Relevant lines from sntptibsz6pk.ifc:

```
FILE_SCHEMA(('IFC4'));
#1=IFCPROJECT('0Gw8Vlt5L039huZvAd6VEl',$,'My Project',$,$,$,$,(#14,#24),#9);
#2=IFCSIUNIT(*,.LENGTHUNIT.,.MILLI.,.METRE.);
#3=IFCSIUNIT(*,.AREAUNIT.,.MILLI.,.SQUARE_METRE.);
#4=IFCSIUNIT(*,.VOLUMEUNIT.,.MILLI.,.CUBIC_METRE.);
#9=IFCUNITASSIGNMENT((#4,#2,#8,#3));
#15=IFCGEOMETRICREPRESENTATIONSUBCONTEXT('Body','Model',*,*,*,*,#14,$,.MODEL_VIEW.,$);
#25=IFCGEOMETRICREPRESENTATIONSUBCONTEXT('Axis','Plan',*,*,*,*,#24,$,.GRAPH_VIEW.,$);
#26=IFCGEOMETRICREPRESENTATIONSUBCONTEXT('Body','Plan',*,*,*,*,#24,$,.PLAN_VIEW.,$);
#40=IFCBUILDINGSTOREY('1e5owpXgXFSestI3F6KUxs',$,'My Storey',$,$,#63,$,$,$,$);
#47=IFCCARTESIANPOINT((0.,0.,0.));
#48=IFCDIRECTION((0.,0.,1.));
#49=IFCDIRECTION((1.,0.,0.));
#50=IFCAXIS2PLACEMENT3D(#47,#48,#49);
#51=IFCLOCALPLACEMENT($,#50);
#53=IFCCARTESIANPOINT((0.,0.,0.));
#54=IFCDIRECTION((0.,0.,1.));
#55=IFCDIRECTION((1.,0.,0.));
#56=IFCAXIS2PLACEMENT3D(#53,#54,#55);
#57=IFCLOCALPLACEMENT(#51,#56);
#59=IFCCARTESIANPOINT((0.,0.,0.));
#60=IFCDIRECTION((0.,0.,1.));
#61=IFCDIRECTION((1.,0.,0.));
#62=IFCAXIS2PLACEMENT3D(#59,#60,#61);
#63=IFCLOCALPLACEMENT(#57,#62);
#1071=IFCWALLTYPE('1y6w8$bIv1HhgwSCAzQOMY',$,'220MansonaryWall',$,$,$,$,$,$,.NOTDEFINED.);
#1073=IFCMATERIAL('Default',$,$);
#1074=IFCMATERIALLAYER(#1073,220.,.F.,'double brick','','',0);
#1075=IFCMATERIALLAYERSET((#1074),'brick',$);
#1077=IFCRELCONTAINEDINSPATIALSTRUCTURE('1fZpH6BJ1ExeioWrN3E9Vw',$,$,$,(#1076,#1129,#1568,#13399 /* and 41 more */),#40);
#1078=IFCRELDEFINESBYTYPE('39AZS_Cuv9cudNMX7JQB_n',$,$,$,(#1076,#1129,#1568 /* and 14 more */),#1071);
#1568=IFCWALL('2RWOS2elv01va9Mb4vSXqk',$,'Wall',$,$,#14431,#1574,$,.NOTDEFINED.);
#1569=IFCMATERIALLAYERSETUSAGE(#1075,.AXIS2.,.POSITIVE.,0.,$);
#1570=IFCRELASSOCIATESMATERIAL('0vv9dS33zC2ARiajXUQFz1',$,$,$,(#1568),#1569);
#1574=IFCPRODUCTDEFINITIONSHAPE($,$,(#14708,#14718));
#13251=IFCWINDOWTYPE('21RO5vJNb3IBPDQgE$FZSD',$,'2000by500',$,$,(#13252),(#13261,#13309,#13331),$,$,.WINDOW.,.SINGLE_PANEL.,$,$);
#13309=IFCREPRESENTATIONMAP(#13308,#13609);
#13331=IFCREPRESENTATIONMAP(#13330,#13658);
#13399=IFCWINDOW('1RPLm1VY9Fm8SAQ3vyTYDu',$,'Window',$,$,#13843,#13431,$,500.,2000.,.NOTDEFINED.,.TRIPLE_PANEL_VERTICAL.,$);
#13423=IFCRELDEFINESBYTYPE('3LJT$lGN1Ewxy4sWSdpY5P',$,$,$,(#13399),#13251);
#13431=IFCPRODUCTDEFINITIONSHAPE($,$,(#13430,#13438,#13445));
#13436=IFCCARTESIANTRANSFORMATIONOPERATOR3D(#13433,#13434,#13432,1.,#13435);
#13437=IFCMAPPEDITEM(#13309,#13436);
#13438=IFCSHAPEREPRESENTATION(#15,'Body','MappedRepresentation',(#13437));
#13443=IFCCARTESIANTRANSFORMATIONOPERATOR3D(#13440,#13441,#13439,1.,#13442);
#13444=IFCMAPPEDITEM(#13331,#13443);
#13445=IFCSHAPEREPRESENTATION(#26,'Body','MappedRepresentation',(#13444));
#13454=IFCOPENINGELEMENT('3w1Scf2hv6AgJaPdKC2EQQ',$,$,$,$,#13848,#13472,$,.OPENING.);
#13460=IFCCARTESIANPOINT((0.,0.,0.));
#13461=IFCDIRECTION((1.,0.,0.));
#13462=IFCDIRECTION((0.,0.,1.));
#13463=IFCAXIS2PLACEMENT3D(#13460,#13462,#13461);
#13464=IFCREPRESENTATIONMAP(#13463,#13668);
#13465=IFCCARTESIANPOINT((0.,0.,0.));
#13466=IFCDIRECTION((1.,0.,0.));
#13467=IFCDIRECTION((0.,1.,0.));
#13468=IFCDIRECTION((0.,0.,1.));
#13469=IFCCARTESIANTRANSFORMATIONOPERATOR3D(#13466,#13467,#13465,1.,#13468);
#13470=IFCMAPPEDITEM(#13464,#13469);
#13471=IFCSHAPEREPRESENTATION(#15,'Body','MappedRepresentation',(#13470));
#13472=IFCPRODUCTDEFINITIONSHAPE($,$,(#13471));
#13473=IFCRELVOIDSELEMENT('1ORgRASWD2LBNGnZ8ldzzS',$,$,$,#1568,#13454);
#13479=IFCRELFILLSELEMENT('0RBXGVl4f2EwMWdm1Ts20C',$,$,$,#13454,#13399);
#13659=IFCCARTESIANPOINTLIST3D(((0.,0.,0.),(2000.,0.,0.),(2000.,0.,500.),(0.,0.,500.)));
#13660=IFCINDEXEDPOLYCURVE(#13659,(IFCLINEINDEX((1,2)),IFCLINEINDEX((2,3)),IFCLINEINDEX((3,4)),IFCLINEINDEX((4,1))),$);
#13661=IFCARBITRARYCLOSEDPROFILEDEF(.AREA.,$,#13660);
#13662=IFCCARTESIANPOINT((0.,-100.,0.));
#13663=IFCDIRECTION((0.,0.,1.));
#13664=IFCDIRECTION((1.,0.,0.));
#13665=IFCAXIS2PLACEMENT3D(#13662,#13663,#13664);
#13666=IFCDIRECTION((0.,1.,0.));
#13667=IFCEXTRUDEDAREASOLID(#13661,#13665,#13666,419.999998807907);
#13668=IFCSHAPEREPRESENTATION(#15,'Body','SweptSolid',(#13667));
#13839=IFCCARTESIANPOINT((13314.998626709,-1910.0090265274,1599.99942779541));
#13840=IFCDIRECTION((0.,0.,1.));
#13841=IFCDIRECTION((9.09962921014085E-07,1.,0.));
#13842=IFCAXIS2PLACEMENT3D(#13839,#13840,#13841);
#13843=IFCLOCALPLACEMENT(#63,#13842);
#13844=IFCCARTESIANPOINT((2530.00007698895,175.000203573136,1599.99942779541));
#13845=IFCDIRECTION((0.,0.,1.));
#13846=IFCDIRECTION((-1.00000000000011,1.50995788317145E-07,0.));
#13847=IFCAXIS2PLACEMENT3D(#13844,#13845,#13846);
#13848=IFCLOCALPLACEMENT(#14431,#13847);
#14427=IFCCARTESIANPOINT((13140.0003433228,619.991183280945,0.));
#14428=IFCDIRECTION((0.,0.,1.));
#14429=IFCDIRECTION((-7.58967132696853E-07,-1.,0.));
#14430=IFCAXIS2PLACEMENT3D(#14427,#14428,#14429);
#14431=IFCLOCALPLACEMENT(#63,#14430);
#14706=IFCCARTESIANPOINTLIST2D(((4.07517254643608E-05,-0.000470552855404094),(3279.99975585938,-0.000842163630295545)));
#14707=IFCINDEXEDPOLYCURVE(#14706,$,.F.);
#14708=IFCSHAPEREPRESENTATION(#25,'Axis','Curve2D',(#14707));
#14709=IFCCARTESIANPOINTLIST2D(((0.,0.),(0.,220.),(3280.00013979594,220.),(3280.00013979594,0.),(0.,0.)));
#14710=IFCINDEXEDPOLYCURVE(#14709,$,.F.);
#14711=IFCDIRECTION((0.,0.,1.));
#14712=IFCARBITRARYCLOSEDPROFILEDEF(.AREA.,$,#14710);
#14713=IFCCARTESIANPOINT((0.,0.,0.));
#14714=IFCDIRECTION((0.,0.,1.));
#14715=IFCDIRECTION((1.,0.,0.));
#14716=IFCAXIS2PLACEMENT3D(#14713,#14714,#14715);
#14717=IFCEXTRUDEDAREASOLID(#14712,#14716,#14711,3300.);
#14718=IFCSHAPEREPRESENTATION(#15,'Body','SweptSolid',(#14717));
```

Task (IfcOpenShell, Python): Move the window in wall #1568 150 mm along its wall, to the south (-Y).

```python
import ifcopenshell
import ifcopenshell.api.geometry
import ifcopenshell.util.placement
import ifcopenshell.util.unit

model = ifcopenshell.open("sntptibsz6pk.ifc")
unit_scale = ifcopenshell.util.unit.calculate_unit_scale(model)

window = model.by_guid("1RPLm1VY9Fm8SAQ3vyTYDu")
opening = window.FillsVoids[0].RelatingOpeningElement
wall = opening.VoidsElements[0].RelatingBuildingElement

wall_matrix = ifcopenshell.util.placement.get_local_placement(wall.ObjectPlacement)
shift = wall_matrix[:3, 0] * 0.15 / unit_scale
before = ifcopenshell.util.placement.get_local_placement(window.ObjectPlacement)[:3, 3].copy()

# The window is not placed relative to its opening, so move both.
for product in (opening, window):
    matrix = ifcopenshell.util.placement.get_local_placement(product.ObjectPlacement)
    matrix[:3, 3] += shift
    ifcopenshell.api.geometry.edit_object_placement(model, product=product, matrix=matrix, is_si=False)

after = ifcopenshell.util.placement.get_local_placement(window.ObjectPlacement)[:3, 3]
print("window moved by", (after - before).round(3) + 0.0)

model.write("sntptibsz6pk_edited.ifc")
```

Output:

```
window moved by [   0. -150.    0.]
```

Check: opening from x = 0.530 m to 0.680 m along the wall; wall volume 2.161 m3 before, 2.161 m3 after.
